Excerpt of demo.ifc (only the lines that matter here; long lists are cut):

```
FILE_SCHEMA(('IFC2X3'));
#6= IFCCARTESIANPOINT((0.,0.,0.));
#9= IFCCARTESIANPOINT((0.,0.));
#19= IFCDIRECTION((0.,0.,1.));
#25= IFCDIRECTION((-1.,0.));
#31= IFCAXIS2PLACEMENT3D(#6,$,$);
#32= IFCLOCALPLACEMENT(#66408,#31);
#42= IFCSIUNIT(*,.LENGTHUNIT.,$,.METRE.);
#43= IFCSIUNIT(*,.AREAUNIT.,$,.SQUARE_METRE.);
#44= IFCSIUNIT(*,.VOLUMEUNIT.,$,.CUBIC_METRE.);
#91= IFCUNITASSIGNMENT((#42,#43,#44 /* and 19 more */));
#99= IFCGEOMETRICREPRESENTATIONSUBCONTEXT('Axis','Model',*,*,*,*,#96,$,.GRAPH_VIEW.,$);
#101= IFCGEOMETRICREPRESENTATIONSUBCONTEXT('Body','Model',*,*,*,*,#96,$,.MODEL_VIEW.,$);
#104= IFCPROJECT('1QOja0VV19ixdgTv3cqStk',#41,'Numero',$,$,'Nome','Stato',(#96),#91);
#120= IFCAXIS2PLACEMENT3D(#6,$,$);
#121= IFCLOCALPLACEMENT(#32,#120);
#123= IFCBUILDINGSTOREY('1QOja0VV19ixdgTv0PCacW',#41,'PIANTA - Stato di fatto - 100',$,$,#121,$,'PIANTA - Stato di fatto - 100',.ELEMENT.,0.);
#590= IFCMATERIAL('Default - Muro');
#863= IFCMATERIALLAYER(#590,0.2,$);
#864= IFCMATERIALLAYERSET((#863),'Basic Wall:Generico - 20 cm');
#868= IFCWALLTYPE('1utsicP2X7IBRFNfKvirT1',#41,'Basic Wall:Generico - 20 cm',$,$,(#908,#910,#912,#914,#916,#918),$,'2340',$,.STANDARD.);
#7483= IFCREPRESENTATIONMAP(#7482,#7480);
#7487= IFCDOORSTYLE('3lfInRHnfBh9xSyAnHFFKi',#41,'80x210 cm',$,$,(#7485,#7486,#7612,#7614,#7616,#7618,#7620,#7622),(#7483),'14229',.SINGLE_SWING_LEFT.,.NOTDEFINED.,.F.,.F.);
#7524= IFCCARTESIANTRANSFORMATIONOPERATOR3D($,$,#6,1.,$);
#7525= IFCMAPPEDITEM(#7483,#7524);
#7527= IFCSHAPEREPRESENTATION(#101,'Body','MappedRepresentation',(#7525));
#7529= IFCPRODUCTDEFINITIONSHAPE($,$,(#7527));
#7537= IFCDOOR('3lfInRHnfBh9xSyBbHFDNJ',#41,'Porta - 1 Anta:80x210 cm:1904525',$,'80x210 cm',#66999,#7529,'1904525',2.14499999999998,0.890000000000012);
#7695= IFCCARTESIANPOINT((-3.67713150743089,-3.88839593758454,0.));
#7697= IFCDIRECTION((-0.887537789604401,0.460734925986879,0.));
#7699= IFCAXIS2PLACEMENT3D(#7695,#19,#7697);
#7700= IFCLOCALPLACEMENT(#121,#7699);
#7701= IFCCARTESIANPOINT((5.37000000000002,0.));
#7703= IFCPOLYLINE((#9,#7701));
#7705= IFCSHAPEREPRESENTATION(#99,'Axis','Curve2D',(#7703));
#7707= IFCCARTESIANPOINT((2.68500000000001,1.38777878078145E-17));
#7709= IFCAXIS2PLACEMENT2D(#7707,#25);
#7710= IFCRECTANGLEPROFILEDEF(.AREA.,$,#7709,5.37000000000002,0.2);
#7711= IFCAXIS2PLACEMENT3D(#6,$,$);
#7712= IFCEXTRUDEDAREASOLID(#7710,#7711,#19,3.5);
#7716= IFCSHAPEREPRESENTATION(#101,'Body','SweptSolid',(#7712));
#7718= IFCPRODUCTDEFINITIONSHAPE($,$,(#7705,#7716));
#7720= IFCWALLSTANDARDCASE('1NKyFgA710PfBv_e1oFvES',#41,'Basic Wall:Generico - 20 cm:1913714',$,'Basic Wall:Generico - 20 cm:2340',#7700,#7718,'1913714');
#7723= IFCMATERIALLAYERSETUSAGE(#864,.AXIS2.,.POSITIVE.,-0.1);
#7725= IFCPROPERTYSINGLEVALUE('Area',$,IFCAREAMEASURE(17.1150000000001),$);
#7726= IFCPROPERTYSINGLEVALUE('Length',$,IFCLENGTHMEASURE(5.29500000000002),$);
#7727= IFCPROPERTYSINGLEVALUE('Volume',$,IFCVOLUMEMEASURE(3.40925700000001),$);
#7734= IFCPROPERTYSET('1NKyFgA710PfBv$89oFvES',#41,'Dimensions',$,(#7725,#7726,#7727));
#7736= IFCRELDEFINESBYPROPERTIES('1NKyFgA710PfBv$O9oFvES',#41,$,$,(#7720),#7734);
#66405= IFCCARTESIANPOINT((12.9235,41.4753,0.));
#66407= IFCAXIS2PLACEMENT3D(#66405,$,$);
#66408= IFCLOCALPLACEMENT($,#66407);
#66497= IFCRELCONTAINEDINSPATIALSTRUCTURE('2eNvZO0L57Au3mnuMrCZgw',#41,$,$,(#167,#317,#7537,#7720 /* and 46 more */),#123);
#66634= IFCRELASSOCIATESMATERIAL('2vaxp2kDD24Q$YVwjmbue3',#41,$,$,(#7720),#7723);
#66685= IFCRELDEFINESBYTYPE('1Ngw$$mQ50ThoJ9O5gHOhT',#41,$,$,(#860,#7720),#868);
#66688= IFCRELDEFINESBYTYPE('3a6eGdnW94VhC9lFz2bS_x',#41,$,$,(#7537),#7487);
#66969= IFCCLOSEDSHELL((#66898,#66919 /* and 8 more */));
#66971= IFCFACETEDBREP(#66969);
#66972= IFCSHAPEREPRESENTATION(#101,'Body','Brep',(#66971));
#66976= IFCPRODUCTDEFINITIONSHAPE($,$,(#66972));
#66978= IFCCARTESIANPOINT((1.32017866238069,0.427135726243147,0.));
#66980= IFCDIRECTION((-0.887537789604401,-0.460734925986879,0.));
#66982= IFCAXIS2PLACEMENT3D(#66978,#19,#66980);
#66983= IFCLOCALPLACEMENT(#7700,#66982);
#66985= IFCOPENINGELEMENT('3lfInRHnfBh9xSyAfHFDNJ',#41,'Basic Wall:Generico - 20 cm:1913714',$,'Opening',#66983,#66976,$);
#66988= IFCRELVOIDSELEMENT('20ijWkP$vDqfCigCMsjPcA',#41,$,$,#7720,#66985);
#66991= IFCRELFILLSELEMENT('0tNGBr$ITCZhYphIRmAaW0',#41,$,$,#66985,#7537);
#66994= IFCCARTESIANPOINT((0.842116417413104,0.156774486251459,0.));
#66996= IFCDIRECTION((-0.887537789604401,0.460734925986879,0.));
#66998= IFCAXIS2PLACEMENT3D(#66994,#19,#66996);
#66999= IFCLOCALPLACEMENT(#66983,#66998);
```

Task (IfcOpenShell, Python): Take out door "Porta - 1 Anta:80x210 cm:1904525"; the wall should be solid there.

```python
import ifcopenshell
import ifcopenshell.api.feature
import ifcopenshell.api.pset
import ifcopenshell.api.root
import ifcopenshell.geom
import ifcopenshell.util.element
import ifcopenshell.util.shape
import ifcopenshell.util.unit

model = ifcopenshell.open("demo.ifc")
area_scale = ifcopenshell.util.unit.calculate_unit_scale(model, "AREAUNIT")
volume_scale = ifcopenshell.util.unit.calculate_unit_scale(model, "VOLUMEUNIT")
settings = ifcopenshell.geom.settings()


def volume(element):
    """Net volume in cubic metres, openings subtracted."""
    shape = ifcopenshell.geom.create_shape(settings, element)
    return ifcopenshell.util.shape.get_volume(shape.geometry)


door = model.by_id(7537)
opening = door.FillsVoids[0].RelatingOpeningElement
wall = opening.VoidsElements[0].RelatingBuildingElement
before = volume(wall)

ifcopenshell.api.root.remove_product(model, product=door)
ifcopenshell.api.feature.remove_feature(model, feature=opening)

after = volume(wall)
thickness = 0.2  # wall thickness in metres

# Update the wall's stored quantities.
pset = model.by_id(ifcopenshell.util.element.get_pset(wall, "Dimensions", should_inherit=False)["id"])
ifcopenshell.api.pset.edit_pset(model, pset=pset, properties={
    "Area": model.create_entity("IfcAreaMeasure", after / thickness / area_scale),
    "Volume": model.create_entity("IfcVolumeMeasure", after / volume_scale),
})

print(f"wall volume {before:.3f} -> {after:.3f} m3")

model.write("demo_edited.ifc")
```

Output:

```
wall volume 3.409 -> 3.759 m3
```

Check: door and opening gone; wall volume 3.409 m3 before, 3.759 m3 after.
